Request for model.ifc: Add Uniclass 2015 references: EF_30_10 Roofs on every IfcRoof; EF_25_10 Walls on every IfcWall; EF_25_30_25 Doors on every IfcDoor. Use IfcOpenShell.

First a look at what the model holds.

```python
import ifcopenshell

model = ifcopenshell.open("model.ifc")
print(model.schema)
print("classifications:", [c.Name for c in model.by_type("IfcClassification")])
for ifc_class in ("IfcDoor", "IfcRoof", "IfcStair", "IfcWall", "IfcWindow"):
    print(ifc_class, len(model.by_type(ifc_class)))
```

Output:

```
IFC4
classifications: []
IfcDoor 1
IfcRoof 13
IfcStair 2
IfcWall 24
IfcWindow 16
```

```python
import ifcopenshell
import ifcopenshell.api.classification

model = ifcopenshell.open("model.ifc")

system = ifcopenshell.api.classification.add_classification(model, classification="Uniclass 2015")

codes = {
    "IfcRoof": ("EF_30_10", "Roofs"),
    "IfcWall": ("EF_25_10", "Walls"),
    "IfcDoor": ("EF_25_30_25", "Doors"),
}
for ifc_class, (code, name) in codes.items():
    products = model.by_type(ifc_class)
    ifcopenshell.api.classification.add_reference(
        model, products=products, classification=system, identification=code, name=name
    )
    print(code, len(products))

model.write("model_rev.ifc")
```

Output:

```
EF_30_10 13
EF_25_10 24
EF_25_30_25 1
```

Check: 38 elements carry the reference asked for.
